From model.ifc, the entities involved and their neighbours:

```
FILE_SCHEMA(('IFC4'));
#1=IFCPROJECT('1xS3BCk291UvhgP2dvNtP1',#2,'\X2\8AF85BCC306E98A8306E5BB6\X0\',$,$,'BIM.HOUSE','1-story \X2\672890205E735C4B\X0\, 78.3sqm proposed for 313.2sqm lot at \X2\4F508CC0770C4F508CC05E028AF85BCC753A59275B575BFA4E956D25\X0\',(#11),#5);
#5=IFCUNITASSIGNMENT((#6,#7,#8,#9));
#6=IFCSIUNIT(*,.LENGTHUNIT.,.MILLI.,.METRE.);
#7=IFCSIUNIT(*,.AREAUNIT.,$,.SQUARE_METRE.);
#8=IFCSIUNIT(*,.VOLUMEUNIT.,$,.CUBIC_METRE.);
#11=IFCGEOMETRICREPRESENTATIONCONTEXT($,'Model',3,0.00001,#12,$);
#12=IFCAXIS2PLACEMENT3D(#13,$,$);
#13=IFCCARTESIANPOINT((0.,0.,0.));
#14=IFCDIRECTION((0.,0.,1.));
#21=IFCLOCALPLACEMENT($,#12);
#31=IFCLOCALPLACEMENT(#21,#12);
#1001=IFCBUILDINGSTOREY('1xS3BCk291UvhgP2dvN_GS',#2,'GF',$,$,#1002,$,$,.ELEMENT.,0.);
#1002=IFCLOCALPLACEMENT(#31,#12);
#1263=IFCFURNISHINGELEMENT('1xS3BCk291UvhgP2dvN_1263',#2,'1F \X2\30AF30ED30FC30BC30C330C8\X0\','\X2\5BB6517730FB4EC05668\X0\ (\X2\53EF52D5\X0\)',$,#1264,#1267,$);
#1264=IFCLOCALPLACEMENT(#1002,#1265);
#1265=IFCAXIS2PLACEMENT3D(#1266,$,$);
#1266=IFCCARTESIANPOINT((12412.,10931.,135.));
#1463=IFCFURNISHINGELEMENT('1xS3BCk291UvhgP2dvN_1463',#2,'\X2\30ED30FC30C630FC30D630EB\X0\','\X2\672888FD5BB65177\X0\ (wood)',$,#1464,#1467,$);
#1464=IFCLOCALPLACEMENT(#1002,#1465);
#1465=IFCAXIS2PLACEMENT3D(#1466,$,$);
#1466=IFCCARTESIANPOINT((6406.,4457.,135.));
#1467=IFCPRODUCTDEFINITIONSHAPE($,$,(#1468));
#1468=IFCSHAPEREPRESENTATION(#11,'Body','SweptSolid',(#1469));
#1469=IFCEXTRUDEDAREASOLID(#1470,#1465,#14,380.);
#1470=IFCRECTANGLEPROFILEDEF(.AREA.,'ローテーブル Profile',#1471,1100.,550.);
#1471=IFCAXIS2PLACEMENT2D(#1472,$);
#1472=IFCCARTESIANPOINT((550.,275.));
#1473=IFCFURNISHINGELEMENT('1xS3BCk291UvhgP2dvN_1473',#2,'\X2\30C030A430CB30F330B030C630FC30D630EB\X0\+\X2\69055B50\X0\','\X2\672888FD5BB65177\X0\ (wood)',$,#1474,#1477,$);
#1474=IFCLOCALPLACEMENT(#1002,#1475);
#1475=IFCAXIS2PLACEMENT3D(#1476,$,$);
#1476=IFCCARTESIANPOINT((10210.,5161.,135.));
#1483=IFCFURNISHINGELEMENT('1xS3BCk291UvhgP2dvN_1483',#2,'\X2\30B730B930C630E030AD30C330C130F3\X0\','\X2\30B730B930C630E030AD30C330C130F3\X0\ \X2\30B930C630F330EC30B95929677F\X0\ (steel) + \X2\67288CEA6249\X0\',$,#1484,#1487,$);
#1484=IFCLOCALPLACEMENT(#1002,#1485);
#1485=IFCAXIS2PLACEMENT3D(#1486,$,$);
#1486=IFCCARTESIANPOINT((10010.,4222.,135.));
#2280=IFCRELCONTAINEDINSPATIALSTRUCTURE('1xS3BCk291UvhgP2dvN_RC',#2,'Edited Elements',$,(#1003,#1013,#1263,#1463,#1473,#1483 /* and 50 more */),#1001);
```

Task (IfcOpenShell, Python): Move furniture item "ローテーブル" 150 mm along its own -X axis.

```python
import ifcopenshell
import ifcopenshell.api.geometry
import ifcopenshell.util.placement
import ifcopenshell.util.unit

model = ifcopenshell.open("model.ifc")
unit_scale = ifcopenshell.util.unit.calculate_unit_scale(model)

item = model.by_id(1463)
matrix = ifcopenshell.util.placement.get_local_placement(item.ObjectPlacement)
matrix[:3, 3] -= matrix[:3, 0] * 0.15 / unit_scale
ifcopenshell.api.geometry.edit_object_placement(model, product=item, matrix=matrix, is_si=False)

print(ifcopenshell.util.placement.get_local_placement(item.ObjectPlacement).round(3) + 0.0)

model.write("model_rev.ifc")
```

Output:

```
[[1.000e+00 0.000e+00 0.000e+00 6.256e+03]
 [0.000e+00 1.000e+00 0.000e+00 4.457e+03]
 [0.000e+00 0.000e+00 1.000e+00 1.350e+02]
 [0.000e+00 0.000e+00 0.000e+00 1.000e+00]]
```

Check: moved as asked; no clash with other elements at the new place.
